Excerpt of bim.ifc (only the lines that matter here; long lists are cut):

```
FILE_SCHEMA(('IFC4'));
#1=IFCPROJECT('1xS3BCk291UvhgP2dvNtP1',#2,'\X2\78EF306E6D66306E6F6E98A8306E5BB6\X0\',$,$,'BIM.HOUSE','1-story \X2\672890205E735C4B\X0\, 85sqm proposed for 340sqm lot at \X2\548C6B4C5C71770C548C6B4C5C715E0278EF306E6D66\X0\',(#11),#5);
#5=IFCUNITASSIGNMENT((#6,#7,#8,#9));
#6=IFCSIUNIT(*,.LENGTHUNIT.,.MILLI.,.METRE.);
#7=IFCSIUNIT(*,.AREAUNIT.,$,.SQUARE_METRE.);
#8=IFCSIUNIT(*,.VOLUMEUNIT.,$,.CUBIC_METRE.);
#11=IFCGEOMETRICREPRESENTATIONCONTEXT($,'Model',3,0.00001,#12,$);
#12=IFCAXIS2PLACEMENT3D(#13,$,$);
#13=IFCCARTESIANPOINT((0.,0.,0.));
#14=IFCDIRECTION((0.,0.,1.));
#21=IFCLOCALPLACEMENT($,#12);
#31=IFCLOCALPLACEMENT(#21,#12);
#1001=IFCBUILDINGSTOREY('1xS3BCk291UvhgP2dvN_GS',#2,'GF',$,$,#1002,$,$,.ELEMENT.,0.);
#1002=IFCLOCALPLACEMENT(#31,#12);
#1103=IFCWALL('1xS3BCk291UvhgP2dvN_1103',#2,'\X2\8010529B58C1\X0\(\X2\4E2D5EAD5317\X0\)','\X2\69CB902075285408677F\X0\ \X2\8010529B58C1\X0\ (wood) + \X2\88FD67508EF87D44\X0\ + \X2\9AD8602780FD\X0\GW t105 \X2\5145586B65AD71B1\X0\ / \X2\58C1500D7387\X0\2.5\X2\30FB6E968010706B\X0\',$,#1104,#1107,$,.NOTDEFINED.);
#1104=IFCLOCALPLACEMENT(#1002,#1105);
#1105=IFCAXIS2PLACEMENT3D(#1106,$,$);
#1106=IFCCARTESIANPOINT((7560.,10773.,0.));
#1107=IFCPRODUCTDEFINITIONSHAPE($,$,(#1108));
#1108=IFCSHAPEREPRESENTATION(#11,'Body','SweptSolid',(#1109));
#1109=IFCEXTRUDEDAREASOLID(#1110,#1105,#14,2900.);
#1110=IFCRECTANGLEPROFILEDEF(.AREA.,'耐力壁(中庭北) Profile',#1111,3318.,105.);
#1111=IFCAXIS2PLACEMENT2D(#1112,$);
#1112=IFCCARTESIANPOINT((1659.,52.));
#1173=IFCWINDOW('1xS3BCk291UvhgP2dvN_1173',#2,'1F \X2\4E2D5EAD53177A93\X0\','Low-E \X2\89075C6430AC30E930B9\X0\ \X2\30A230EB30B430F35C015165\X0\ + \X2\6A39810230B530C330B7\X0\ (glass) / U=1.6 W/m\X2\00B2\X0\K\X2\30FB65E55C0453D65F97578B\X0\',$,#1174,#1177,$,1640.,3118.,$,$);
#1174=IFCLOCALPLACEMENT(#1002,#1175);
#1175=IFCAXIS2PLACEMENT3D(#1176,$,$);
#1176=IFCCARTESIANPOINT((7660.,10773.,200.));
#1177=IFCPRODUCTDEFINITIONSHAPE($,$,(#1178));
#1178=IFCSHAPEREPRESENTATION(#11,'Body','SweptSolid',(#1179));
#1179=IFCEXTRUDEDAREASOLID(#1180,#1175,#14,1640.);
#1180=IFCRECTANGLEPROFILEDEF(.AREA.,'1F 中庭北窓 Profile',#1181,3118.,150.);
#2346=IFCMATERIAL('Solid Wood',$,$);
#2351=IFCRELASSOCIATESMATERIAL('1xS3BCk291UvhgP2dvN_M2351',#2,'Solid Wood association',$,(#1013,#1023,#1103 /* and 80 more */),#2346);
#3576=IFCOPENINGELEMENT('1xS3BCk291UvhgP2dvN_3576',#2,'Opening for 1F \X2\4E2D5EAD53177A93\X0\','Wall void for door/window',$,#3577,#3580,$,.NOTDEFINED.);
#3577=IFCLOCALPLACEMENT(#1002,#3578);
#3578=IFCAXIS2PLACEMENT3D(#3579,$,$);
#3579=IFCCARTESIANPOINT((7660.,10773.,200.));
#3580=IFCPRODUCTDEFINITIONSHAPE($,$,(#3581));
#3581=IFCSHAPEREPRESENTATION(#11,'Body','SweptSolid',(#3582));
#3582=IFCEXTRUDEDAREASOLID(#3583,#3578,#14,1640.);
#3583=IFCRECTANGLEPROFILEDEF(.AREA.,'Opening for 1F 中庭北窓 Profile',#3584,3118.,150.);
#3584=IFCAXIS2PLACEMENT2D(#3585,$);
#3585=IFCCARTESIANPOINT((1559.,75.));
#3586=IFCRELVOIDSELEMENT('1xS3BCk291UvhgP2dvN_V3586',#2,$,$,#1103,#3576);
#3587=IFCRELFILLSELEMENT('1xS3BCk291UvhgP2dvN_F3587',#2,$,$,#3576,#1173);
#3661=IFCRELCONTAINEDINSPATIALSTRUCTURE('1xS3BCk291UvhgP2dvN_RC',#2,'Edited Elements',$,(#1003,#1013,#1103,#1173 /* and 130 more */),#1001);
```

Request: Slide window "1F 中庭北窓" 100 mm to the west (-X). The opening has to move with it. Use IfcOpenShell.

```python
import ifcopenshell
import ifcopenshell.api.geometry
import ifcopenshell.util.placement

model = ifcopenshell.open("bim.ifc")

window = model.by_guid("1xS3BCk291UvhgP2dvN_1173")
opening = window.FillsVoids[0].RelatingOpeningElement
wall = opening.VoidsElements[0].RelatingBuildingElement

wall_matrix = ifcopenshell.util.placement.get_local_placement(wall.ObjectPlacement)
shift = wall_matrix[:3, 0] * -100.0
before = ifcopenshell.util.placement.get_local_placement(window.ObjectPlacement)[:3, 3].copy()

# The window is not placed relative to its opening, so move both.
for product in (opening, window):
    matrix = ifcopenshell.util.placement.get_local_placement(product.ObjectPlacement)
    matrix[:3, 3] += shift
    ifcopenshell.api.geometry.edit_object_placement(model, product=product, matrix=matrix, is_si=False)

after = ifcopenshell.util.placement.get_local_placement(window.ObjectPlacement)[:3, 3]
print("window moved by", (after - before).round(3) + 0.0)

model.write("bim_rev.ifc")
```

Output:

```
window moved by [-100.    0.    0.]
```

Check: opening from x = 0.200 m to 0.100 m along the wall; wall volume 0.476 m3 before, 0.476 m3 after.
